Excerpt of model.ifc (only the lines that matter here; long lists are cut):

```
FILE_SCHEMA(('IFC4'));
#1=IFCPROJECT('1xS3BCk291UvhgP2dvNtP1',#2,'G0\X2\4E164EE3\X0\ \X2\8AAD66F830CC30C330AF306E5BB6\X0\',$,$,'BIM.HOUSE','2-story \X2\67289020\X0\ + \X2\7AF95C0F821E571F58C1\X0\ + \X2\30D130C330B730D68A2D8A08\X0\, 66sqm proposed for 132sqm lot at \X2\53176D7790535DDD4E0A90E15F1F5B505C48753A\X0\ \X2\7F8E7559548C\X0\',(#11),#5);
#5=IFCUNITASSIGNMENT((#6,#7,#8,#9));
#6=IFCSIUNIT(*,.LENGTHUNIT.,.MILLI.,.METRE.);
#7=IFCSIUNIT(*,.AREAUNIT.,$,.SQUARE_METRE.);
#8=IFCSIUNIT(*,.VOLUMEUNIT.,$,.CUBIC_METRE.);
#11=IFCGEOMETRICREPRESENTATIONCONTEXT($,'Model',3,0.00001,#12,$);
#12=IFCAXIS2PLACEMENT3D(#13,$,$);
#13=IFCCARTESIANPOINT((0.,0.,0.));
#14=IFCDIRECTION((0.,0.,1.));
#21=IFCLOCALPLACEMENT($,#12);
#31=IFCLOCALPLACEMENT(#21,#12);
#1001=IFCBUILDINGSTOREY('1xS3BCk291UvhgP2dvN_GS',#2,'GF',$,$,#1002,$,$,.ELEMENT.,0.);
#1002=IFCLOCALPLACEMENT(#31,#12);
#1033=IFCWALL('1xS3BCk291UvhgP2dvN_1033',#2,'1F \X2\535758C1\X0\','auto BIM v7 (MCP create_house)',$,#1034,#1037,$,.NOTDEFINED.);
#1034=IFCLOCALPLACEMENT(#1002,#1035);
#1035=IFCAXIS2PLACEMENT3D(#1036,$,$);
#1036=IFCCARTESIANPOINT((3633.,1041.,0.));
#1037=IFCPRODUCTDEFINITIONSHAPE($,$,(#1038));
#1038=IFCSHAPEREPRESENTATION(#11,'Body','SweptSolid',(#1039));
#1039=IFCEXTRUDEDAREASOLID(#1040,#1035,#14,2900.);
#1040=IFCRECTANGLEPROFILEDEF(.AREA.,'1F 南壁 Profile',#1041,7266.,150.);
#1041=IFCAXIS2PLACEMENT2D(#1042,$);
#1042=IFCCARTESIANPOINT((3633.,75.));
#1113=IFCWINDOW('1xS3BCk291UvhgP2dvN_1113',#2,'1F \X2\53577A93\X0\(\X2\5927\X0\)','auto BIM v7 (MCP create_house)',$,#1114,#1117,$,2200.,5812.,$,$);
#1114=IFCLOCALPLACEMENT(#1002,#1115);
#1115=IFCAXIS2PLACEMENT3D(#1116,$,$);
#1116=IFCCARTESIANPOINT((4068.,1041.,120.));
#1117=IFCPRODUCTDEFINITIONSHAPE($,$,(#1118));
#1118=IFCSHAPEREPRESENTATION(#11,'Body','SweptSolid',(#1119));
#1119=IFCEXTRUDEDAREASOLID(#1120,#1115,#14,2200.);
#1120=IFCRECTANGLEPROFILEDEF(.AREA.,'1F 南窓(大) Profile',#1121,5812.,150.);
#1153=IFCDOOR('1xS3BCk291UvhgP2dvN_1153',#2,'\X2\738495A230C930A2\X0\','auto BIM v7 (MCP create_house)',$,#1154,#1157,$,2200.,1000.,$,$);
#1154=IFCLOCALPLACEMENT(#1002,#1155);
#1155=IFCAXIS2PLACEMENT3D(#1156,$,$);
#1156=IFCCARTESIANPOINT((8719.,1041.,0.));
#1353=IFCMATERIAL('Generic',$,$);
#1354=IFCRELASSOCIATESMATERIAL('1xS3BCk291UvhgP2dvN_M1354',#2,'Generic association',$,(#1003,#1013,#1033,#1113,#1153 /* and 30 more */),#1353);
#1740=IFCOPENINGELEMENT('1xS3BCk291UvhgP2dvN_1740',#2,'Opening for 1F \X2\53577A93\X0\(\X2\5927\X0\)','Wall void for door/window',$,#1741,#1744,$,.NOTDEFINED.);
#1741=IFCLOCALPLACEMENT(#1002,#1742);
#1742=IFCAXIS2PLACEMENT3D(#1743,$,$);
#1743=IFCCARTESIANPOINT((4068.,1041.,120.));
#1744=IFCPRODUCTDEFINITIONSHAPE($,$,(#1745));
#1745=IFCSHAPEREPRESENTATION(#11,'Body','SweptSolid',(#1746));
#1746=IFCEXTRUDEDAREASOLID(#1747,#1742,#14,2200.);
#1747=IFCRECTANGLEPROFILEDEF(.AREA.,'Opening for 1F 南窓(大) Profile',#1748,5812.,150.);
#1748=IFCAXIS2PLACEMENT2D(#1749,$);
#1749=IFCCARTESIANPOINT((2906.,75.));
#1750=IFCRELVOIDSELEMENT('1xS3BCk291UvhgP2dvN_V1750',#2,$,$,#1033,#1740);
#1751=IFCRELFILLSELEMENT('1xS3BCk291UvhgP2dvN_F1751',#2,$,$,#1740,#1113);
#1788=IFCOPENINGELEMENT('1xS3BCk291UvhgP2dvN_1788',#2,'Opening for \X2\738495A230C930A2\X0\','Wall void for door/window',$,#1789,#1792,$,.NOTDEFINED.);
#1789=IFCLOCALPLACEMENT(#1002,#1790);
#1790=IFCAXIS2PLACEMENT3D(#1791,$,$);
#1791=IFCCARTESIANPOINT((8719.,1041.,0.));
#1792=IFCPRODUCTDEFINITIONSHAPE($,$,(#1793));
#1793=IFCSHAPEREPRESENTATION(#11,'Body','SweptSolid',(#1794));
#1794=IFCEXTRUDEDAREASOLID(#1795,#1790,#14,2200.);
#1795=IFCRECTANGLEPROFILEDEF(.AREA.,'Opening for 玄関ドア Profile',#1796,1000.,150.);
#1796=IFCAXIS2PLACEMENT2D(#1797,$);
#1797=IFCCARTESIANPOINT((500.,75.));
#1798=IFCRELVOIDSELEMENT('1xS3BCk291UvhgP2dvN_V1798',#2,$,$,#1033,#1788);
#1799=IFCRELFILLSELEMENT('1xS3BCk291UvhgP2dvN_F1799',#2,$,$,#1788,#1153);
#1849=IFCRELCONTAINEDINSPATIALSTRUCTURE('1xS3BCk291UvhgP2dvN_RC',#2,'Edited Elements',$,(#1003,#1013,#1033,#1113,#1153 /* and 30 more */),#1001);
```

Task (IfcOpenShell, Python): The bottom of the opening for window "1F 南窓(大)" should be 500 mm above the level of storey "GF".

```python
import numpy as np
import ifcopenshell
import ifcopenshell.api.geometry
import ifcopenshell.geom
import ifcopenshell.util.element
import ifcopenshell.util.placement
import ifcopenshell.util.shape
import ifcopenshell.util.unit

model = ifcopenshell.open("model.ifc")
unit_scale = ifcopenshell.util.unit.calculate_unit_scale(model)

window = model.by_guid("1xS3BCk291UvhgP2dvN_1113")
opening = window.FillsVoids[0].RelatingOpeningElement
storey = ifcopenshell.util.element.get_container(window, ifc_class="IfcBuildingStorey")
level = ifcopenshell.util.placement.get_local_placement(storey.ObjectPlacement)[2, 3]

# The opening's origin need not be at the sill, so measure its lowest point.
shape = ifcopenshell.geom.create_shape(ifcopenshell.geom.settings(), opening)
bottom = ifcopenshell.util.shape.get_shape_bottom_elevation(shape, shape.geometry) / unit_scale
dz = level + 0.5 / unit_scale - bottom

shift = np.array([0.0, 0.0, dz])
# The window is not placed relative to its opening, so move both.
for product in (opening, window):
    matrix = ifcopenshell.util.placement.get_local_placement(product.ObjectPlacement)
    matrix[:3, 3] += shift
    ifcopenshell.api.geometry.edit_object_placement(model, product=product, matrix=matrix, is_si=False)

print(f"moved by {dz * unit_scale:+.3f} m")

model.write("model_edited.ifc")
```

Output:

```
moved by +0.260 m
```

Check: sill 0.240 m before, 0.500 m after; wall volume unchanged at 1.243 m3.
